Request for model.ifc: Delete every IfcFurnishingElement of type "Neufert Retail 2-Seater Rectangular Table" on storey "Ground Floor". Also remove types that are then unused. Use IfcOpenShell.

First a look at what the model holds.

```python
import ifcopenshell
import ifcopenshell.util.element

model = ifcopenshell.open("model.ifc")
print(model.schema)
storey = next(s for s in model.by_type("IfcBuildingStorey") if s.Name == "Ground Floor")
furniture = [e for e in ifcopenshell.util.element.get_decomposition(storey) if e.is_a("IfcFurnishingElement")]
seen = {}
for e in furniture:
    element_type = ifcopenshell.util.element.get_type(e)
    name = element_type.Name if element_type not in (None, e) else None
    seen[name] = seen.get(name, 0) + 1
for name, count in sorted(seen.items(), key=str):
    print(count, "x", name)
```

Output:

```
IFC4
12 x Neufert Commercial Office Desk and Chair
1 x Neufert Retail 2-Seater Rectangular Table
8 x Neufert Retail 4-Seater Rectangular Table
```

```python
import ifcopenshell
import ifcopenshell.api.root
import ifcopenshell.util.element

model = ifcopenshell.open("model.ifc")

storey = next(s for s in model.by_type("IfcBuildingStorey") if s.Name == "Ground Floor")
furniture = [e for e in ifcopenshell.util.element.get_decomposition(storey) if e.is_a("IfcFurnishingElement")]
targets = [e for e in furniture if (t := ifcopenshell.util.element.get_type(e)) not in (None, e) and t.Name == "Neufert Retail 2-Seater Rectangular Table"]
types = {ifcopenshell.util.element.get_type(e) for e in targets} - {None, *targets}

for e in targets:
    ifcopenshell.api.root.remove_product(model, product=e)
print(len(targets), "removed")

unused = [t for t in types if not ifcopenshell.util.element.get_types(t)]
for t in unused:
    ifcopenshell.api.root.remove_product(model, product=t)
print(len(unused), "unused types removed")

model.write("model_v2.ifc")
```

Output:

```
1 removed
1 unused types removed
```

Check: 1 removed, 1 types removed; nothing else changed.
